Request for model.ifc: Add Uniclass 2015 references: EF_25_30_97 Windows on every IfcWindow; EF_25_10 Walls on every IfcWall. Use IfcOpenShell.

First a look at what the model holds.

```python
import ifcopenshell

model = ifcopenshell.open("model.ifc")
print(model.schema)
print("classifications:", [c.Name for c in model.by_type("IfcClassification")])
for ifc_class in ("IfcDoor", "IfcRoof", "IfcStair", "IfcWall", "IfcWindow"):
    print(ifc_class, len(model.by_type(ifc_class)))
```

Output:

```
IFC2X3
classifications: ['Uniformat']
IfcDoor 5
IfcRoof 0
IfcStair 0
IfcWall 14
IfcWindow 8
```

```python
import ifcopenshell
import ifcopenshell.api.classification

model = ifcopenshell.open("model.ifc")

# IFC2X3 requires Source and Edition and has no link from the project to the system.
system = model.create_entity("IfcClassification", Source="NBS", Edition="2015", Name="Uniclass 2015")

codes = {
    "IfcWindow": ("EF_25_30_97", "Windows"),
    "IfcWall": ("EF_25_10", "Walls"),
}
for ifc_class, (code, name) in codes.items():
    products = model.by_type(ifc_class)
    ifcopenshell.api.classification.add_reference(
        model, products=products, classification=system, identification=code, name=name
    )
    print(code, len(products))

model.write("model_v2.ifc")
```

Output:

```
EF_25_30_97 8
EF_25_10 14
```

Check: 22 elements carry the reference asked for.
